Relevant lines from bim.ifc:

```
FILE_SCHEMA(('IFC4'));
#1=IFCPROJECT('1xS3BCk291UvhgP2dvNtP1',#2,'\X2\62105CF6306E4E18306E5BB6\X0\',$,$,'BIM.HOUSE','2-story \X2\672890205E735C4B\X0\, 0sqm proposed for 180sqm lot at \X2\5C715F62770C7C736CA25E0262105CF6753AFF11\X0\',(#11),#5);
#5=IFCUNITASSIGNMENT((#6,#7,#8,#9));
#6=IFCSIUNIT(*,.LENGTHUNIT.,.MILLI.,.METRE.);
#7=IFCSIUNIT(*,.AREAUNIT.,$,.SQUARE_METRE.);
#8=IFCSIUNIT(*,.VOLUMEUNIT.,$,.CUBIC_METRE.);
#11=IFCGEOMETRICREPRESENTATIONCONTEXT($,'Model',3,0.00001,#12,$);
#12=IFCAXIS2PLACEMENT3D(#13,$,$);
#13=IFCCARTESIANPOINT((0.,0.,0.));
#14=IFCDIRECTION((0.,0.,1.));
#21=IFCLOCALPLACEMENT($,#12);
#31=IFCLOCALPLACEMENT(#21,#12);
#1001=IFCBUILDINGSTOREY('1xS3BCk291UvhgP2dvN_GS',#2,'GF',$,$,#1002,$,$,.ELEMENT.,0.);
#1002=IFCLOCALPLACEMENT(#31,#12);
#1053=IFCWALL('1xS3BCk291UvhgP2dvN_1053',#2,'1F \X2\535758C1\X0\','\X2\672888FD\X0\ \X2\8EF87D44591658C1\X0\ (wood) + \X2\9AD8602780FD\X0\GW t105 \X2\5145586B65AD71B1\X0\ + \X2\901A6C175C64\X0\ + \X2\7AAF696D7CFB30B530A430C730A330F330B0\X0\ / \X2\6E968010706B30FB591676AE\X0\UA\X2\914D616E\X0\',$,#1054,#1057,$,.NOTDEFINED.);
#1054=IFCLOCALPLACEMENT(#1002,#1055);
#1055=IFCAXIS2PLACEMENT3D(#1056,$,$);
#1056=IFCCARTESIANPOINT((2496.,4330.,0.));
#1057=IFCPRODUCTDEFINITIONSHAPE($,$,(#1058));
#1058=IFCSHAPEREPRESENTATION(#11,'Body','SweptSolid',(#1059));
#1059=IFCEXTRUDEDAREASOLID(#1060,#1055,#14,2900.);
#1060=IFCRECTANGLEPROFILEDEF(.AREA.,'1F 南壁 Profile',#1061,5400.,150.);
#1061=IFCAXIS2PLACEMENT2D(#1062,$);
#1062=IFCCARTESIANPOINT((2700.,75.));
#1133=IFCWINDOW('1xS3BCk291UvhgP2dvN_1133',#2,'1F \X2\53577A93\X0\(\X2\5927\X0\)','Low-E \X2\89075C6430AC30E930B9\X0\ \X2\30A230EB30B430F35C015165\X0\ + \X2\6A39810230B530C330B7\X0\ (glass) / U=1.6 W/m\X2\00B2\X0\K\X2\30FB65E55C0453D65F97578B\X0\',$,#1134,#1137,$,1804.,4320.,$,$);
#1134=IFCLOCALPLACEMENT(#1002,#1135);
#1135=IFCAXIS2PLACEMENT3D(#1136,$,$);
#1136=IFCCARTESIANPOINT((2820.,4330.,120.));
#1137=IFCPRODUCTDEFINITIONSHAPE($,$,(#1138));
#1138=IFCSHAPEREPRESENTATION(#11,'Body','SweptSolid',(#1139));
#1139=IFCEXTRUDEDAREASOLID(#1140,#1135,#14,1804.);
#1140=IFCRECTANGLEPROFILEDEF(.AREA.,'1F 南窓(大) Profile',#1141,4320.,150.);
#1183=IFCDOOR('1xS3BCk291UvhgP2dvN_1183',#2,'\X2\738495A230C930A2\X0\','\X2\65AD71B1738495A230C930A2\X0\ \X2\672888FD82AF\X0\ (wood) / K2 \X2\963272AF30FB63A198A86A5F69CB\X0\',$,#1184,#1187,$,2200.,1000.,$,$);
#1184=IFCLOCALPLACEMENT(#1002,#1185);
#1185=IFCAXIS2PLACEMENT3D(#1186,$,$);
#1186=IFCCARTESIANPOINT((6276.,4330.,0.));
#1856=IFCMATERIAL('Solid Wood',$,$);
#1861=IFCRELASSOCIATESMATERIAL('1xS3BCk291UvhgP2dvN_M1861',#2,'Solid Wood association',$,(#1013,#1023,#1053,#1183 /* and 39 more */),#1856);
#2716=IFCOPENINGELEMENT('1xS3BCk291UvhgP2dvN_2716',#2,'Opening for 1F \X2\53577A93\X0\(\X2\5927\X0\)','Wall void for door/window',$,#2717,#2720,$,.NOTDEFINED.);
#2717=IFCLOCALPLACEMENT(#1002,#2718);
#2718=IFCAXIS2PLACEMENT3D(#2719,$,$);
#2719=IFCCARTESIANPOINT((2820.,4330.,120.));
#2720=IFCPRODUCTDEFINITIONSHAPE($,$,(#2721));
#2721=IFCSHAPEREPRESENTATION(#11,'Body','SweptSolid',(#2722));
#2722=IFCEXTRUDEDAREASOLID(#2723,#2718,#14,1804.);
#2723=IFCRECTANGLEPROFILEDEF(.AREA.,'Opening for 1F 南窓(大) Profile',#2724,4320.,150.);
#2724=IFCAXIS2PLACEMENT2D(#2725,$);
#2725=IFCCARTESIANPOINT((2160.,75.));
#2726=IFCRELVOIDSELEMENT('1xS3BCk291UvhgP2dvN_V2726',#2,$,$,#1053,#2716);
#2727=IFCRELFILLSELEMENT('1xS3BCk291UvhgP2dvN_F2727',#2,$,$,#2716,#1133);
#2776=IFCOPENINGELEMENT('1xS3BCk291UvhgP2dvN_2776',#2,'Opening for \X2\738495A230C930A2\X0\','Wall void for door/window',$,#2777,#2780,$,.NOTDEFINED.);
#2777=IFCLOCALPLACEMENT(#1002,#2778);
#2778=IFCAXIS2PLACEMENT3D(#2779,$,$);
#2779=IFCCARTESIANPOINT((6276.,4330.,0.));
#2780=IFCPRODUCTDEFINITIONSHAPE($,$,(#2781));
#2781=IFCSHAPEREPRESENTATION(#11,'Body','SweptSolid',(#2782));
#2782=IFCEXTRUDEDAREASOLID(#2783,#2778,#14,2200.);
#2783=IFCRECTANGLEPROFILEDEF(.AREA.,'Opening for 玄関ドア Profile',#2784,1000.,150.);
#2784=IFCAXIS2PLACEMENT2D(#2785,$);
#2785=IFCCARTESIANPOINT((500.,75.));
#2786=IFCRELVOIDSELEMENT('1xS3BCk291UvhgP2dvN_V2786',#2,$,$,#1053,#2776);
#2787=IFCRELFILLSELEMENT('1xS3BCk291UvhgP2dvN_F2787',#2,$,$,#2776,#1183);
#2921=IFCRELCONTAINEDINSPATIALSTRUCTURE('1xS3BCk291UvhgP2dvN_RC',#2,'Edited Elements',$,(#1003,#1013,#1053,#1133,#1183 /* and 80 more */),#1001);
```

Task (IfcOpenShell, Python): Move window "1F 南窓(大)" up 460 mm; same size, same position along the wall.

```python
import numpy as np
import ifcopenshell
import ifcopenshell.api.geometry
import ifcopenshell.util.placement
import ifcopenshell.util.unit

model = ifcopenshell.open("bim.ifc")
unit_scale = ifcopenshell.util.unit.calculate_unit_scale(model)

window = model.by_id(1133)
opening = window.FillsVoids[0].RelatingOpeningElement
dz = 0.46 / unit_scale

shift = np.array([0.0, 0.0, dz])
# The window is not placed relative to its opening, so move both.
for product in (opening, window):
    matrix = ifcopenshell.util.placement.get_local_placement(product.ObjectPlacement)
    matrix[:3, 3] += shift
    ifcopenshell.api.geometry.edit_object_placement(model, product=product, matrix=matrix, is_si=False)

print(f"moved by {dz * unit_scale:+.3f} m")

model.write("bim_edited.ifc")
```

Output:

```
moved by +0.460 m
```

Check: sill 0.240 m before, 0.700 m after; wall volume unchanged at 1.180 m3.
